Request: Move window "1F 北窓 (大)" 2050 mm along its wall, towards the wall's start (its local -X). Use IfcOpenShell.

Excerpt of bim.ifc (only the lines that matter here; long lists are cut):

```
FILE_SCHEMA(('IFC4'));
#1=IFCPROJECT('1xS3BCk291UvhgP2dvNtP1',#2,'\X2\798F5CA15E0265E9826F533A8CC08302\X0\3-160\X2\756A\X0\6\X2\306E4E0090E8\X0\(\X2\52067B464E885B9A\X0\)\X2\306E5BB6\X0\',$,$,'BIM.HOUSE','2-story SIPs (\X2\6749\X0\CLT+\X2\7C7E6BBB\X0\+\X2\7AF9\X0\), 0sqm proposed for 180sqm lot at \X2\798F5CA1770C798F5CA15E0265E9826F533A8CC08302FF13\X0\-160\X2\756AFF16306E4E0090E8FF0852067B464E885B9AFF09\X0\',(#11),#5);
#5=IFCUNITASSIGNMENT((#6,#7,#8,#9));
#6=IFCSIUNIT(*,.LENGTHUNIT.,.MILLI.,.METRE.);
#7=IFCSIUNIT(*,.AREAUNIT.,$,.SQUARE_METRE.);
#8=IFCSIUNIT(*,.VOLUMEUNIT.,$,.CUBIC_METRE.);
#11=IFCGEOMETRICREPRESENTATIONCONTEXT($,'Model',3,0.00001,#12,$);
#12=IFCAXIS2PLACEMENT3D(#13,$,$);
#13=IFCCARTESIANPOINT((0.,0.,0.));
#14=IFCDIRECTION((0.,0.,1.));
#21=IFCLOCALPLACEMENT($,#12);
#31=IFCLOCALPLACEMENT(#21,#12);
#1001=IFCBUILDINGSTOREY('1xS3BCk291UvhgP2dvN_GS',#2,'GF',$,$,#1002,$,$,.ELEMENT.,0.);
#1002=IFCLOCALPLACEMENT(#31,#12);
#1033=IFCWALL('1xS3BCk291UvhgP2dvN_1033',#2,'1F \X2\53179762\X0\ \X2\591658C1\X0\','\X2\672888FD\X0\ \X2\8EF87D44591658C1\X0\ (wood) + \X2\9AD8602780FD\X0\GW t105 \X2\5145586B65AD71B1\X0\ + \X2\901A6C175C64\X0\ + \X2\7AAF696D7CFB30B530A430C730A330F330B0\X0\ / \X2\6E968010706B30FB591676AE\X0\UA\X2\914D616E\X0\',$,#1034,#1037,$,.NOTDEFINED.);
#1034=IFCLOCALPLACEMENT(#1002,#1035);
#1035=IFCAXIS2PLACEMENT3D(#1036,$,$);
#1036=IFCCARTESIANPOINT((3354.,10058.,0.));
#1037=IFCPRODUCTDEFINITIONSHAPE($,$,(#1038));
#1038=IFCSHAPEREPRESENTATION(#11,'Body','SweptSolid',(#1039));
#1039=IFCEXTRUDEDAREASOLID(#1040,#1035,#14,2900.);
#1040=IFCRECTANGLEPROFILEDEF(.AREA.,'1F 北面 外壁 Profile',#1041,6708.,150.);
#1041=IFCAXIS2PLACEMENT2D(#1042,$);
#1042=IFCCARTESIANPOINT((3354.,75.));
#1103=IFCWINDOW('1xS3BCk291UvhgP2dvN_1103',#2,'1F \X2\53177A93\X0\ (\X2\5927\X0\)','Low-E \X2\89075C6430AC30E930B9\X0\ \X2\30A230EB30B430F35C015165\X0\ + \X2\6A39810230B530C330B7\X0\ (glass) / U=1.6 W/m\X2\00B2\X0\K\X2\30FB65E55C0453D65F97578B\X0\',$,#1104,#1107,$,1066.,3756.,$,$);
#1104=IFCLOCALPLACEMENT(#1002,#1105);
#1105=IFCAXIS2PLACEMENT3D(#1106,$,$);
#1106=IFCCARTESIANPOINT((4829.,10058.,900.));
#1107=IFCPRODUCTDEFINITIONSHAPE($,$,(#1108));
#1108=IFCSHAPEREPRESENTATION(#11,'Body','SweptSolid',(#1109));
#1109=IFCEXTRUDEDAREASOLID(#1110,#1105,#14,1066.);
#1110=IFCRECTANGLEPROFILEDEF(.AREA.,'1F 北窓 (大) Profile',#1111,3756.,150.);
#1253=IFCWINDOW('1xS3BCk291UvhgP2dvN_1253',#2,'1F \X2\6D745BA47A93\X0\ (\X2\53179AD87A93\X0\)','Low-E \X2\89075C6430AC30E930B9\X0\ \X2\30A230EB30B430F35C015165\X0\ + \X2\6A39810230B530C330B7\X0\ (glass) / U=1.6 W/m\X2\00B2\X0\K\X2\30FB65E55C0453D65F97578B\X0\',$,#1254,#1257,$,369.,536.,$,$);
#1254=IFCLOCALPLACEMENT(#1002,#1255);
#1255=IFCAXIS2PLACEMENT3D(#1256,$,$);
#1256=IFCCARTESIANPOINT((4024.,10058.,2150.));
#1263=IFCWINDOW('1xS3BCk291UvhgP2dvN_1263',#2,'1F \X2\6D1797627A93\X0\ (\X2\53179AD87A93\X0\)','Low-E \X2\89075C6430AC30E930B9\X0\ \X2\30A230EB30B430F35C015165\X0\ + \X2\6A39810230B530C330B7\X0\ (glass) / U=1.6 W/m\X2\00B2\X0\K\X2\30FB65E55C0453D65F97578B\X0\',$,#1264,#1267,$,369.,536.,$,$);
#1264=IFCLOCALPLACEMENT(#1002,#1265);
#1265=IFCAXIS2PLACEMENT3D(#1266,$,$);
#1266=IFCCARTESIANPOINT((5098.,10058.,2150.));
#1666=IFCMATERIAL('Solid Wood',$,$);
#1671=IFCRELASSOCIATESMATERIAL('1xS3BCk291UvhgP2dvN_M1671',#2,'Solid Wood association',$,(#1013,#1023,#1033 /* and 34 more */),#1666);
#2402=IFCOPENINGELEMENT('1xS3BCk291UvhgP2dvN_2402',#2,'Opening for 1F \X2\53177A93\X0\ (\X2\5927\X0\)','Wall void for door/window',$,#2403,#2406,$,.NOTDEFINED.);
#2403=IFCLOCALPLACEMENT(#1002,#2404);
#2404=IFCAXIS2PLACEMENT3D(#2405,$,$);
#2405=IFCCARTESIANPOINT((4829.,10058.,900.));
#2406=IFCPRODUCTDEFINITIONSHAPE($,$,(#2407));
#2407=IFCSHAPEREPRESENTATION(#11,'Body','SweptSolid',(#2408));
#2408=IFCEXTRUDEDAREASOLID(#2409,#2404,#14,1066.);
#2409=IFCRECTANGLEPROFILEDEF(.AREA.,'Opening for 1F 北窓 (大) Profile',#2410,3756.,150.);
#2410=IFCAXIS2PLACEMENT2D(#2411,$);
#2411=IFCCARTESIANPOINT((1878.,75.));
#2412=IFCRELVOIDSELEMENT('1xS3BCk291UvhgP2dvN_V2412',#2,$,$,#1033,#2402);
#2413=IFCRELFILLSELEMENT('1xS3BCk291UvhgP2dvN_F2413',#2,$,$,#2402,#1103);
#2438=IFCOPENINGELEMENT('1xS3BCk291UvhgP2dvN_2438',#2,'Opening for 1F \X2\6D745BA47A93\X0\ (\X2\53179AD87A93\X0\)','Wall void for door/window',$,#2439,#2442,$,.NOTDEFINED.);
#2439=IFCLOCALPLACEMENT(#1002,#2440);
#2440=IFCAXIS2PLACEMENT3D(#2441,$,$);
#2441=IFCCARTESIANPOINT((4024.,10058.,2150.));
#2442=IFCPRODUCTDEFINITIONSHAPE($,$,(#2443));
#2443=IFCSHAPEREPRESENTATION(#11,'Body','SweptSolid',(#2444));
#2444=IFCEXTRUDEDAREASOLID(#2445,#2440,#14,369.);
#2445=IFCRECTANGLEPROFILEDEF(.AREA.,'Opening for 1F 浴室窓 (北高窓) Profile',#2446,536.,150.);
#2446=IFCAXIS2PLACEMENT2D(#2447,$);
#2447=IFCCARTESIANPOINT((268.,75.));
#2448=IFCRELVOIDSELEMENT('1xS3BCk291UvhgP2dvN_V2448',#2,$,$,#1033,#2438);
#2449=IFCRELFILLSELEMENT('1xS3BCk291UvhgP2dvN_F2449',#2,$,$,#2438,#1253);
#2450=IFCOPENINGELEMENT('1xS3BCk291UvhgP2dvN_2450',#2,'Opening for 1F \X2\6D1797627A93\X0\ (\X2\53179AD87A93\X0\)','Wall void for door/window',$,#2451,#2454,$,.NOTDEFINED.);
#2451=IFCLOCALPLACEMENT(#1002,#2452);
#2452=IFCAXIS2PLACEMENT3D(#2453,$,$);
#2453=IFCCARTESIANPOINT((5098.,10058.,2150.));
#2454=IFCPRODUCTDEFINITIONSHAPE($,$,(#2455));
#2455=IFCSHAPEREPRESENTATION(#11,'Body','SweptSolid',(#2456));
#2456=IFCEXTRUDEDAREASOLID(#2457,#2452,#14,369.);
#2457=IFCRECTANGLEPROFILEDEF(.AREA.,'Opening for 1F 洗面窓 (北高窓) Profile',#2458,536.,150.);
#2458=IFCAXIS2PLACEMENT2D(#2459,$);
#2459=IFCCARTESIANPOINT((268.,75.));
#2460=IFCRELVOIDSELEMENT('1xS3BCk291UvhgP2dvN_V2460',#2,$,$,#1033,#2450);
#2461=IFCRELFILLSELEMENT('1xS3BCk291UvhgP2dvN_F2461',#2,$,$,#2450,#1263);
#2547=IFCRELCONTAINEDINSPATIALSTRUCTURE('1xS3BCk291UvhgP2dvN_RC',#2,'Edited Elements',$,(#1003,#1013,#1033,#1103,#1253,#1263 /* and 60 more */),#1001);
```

```python
import ifcopenshell
import ifcopenshell.api.geometry
import ifcopenshell.util.placement
import ifcopenshell.util.unit

model = ifcopenshell.open("bim.ifc")
unit_scale = ifcopenshell.util.unit.calculate_unit_scale(model)

window = model.by_guid("1xS3BCk291UvhgP2dvN_1103")
opening = window.FillsVoids[0].RelatingOpeningElement
wall = opening.VoidsElements[0].RelatingBuildingElement

wall_matrix = ifcopenshell.util.placement.get_local_placement(wall.ObjectPlacement)
shift = wall_matrix[:3, 0] * -2.05 / unit_scale
before = ifcopenshell.util.placement.get_local_placement(window.ObjectPlacement)[:3, 3].copy()

# The window is not placed relative to its opening, so move both.
for product in (opening, window):
    matrix = ifcopenshell.util.placement.get_local_placement(product.ObjectPlacement)
    matrix[:3, 3] += shift
    ifcopenshell.api.geometry.edit_object_placement(model, product=product, matrix=matrix, is_si=False)

after = ifcopenshell.util.placement.get_local_placement(window.ObjectPlacement)[:3, 3]
print("window moved by", (after - before).round(3) + 0.0)

model.write("bim_updated.ifc")
```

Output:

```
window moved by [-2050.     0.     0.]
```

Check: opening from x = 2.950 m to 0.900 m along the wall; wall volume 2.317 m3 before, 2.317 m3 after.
